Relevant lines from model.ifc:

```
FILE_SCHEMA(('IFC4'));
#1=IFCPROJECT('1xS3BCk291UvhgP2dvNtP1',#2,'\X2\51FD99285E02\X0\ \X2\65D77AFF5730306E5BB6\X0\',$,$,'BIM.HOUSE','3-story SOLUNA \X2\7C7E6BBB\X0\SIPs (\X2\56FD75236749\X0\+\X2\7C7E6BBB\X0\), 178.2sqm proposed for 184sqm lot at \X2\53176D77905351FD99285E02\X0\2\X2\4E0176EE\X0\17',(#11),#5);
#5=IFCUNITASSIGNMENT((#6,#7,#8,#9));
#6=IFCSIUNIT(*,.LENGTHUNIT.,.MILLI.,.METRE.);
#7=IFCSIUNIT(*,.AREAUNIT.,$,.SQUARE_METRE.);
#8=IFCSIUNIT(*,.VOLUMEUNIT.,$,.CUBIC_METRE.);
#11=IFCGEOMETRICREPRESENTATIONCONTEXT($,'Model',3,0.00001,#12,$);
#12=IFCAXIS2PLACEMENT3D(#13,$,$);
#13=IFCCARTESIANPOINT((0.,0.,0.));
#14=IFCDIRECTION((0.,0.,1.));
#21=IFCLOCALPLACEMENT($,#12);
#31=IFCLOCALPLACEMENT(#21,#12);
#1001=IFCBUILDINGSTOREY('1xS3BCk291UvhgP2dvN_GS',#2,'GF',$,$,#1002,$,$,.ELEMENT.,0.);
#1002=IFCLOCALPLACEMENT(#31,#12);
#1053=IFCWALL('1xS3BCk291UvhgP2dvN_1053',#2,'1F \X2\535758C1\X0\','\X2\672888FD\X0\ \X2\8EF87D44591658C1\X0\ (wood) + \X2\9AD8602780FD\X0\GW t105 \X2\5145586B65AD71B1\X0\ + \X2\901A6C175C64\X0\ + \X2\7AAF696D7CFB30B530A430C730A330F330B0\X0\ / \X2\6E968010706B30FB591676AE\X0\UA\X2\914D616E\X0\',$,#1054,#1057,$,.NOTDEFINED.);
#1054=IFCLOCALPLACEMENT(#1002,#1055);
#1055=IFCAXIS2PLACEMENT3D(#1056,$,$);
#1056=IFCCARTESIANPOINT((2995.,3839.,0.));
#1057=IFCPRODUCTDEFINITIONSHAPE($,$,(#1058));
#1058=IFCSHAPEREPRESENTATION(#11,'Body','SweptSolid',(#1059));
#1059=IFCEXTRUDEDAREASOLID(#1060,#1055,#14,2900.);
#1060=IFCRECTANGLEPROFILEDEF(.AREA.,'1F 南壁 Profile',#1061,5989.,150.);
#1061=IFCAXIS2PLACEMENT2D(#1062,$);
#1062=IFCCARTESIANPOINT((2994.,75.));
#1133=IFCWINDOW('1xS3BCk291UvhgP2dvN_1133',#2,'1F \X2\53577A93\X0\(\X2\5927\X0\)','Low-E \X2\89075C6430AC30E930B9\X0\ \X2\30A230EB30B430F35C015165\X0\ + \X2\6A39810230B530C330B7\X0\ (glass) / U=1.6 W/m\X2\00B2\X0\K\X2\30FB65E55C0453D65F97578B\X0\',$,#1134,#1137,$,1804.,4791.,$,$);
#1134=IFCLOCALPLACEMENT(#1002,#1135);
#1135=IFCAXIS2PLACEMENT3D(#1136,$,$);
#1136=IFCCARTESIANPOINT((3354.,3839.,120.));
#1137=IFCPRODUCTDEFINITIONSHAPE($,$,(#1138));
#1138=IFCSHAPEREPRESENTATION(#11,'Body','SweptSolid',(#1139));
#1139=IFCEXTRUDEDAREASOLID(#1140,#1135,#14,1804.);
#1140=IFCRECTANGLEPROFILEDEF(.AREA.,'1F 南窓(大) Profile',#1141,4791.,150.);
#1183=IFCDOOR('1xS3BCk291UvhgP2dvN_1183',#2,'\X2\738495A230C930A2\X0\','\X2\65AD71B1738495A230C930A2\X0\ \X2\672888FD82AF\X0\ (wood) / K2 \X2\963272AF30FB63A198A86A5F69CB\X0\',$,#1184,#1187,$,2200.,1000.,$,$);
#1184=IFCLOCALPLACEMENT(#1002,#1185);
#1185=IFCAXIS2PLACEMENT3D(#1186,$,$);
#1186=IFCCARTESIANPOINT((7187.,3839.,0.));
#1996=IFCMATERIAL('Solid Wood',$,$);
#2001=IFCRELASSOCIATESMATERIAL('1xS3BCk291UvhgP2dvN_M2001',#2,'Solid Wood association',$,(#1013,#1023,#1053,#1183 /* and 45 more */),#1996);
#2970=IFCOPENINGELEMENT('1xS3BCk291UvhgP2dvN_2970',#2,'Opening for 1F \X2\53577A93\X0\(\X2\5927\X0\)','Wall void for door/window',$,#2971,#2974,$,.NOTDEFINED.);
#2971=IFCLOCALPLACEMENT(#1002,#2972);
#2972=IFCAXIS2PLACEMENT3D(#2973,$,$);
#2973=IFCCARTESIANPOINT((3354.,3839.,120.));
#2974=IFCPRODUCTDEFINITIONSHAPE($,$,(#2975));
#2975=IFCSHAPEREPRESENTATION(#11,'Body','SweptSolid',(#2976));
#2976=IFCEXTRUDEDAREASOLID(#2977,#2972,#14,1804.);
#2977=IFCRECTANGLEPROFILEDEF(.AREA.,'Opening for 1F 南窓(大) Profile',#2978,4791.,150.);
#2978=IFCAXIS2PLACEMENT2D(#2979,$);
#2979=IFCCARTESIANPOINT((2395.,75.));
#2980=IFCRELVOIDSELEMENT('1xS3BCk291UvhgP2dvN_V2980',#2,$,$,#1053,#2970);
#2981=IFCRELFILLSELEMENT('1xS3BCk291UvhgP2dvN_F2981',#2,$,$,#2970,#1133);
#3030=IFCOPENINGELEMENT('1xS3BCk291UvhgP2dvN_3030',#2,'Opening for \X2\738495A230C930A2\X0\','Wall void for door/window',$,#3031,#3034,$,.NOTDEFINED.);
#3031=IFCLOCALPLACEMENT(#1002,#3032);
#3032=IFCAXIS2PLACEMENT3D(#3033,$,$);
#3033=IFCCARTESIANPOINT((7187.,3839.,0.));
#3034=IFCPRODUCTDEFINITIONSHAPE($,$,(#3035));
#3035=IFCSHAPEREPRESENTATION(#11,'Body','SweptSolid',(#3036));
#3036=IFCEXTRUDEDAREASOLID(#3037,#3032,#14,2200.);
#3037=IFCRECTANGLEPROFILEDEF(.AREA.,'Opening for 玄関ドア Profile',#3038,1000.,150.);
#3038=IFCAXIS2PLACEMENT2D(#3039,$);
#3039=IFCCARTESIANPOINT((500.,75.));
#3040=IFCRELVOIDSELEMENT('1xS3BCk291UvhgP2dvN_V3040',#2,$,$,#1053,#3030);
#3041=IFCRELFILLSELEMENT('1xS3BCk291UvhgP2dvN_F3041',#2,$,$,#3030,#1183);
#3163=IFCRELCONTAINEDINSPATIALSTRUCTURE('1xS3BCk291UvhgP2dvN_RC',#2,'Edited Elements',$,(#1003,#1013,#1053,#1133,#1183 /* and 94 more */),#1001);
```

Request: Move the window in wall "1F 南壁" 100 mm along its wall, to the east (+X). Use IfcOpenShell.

```python
import ifcopenshell
import ifcopenshell.api.geometry
import ifcopenshell.util.placement

model = ifcopenshell.open("model.ifc")

window = model.by_guid("1xS3BCk291UvhgP2dvN_1133")
opening = window.FillsVoids[0].RelatingOpeningElement
wall = opening.VoidsElements[0].RelatingBuildingElement

wall_matrix = ifcopenshell.util.placement.get_local_placement(wall.ObjectPlacement)
shift = wall_matrix[:3, 0] * 100.0
before = ifcopenshell.util.placement.get_local_placement(window.ObjectPlacement)[:3, 3].copy()

# The window is not placed relative to its opening, so move both.
for product in (opening, window):
    matrix = ifcopenshell.util.placement.get_local_placement(product.ObjectPlacement)
    matrix[:3, 3] += shift
    ifcopenshell.api.geometry.edit_object_placement(model, product=product, matrix=matrix, is_si=False)

after = ifcopenshell.util.placement.get_local_placement(window.ObjectPlacement)[:3, 3]
print("window moved by", (after - before).round(3) + 0.0)

model.write("model_updated.ifc")
```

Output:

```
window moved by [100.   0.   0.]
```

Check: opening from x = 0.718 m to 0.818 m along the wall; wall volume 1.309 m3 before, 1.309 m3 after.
